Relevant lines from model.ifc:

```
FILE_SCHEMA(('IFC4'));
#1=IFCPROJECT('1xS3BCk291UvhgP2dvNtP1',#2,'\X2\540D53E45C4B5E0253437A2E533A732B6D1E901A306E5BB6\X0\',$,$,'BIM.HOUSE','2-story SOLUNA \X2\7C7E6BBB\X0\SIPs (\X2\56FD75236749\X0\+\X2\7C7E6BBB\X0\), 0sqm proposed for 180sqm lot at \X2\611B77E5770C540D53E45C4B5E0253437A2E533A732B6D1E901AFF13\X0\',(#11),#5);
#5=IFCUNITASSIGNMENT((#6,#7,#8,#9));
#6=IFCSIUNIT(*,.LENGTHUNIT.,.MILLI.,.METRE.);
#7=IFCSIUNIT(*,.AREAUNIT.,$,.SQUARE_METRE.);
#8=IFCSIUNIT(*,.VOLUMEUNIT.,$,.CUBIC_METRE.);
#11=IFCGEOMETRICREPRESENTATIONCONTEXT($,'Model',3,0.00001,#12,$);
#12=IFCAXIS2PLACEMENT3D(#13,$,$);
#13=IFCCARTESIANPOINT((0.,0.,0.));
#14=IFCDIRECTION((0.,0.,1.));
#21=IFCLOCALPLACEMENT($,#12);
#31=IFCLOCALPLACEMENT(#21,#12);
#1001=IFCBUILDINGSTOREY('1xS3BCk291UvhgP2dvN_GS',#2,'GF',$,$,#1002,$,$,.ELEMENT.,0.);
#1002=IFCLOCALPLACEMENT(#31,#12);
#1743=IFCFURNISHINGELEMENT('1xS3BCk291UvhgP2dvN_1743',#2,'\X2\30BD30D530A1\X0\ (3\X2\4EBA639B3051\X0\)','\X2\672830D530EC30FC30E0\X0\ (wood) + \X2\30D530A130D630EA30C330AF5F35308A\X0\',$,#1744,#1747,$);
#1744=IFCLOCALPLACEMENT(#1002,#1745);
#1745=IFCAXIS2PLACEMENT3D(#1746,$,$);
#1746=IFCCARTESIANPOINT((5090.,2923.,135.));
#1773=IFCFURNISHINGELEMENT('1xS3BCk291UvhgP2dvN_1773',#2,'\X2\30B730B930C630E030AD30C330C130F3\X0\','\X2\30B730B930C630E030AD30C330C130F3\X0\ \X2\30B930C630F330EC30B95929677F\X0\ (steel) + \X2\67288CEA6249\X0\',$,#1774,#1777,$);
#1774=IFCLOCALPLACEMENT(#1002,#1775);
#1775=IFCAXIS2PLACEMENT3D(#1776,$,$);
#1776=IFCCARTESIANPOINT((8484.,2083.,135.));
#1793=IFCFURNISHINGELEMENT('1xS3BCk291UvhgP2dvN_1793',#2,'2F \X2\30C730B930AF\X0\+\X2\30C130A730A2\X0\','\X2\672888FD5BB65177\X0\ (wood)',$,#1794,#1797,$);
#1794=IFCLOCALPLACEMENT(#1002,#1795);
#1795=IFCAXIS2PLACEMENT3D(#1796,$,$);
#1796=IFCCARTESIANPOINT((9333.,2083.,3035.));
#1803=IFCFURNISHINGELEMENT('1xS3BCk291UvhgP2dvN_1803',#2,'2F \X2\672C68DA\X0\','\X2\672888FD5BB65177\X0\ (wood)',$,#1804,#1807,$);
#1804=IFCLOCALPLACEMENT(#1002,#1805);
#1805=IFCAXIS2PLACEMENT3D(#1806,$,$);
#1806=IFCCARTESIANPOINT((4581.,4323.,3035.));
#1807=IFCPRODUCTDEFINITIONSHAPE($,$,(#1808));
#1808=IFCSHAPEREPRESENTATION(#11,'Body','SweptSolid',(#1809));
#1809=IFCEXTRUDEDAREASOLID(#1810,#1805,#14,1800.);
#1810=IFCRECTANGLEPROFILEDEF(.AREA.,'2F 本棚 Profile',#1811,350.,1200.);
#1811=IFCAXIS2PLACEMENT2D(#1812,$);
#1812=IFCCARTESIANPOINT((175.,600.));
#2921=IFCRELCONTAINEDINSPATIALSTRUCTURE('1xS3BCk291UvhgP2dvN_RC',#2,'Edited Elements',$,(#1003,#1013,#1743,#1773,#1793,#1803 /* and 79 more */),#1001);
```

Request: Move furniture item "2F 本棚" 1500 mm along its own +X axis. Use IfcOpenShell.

```python
import ifcopenshell
import ifcopenshell.api.geometry
import ifcopenshell.util.placement
import ifcopenshell.util.unit

model = ifcopenshell.open("model.ifc")
unit_scale = ifcopenshell.util.unit.calculate_unit_scale(model)

item = model.by_id(1803)
matrix = ifcopenshell.util.placement.get_local_placement(item.ObjectPlacement)
matrix[:3, 3] += matrix[:3, 0] * 1.5 / unit_scale
ifcopenshell.api.geometry.edit_object_placement(model, product=item, matrix=matrix, is_si=False)

print(ifcopenshell.util.placement.get_local_placement(item.ObjectPlacement).round(3) + 0.0)

model.write("model_rev.ifc")
```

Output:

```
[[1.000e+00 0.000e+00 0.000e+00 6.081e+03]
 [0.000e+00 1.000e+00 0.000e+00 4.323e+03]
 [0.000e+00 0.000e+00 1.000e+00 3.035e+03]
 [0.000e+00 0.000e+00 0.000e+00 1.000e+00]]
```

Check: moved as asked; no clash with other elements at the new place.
